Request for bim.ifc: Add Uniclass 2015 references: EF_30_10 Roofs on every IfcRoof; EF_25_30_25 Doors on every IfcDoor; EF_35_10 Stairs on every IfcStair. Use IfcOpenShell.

First a look at what the model holds.

```python
import ifcopenshell

model = ifcopenshell.open("bim.ifc")
print(model.schema)
print("classifications:", [c.Name for c in model.by_type("IfcClassification")])
for ifc_class in ("IfcDoor", "IfcRoof", "IfcStair", "IfcWall", "IfcWindow"):
    print(ifc_class, len(model.by_type(ifc_class)))
```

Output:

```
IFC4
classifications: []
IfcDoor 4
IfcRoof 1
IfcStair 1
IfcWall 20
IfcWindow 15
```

```python
import ifcopenshell
import ifcopenshell.api.classification

model = ifcopenshell.open("bim.ifc")

system = ifcopenshell.api.classification.add_classification(model, classification="Uniclass 2015")

codes = {
    "IfcRoof": ("EF_30_10", "Roofs"),
    "IfcDoor": ("EF_25_30_25", "Doors"),
    "IfcStair": ("EF_35_10", "Stairs"),
}
for ifc_class, (code, name) in codes.items():
    products = model.by_type(ifc_class)
    ifcopenshell.api.classification.add_reference(
        model, products=products, classification=system, identification=code, name=name
    )
    print(code, len(products))

model.write("bim-out.ifc")
```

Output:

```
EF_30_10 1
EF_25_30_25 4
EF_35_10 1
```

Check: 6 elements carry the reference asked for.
